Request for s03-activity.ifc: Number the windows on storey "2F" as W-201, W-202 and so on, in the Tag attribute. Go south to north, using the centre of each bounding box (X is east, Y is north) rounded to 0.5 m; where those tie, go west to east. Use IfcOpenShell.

First a look at what the model holds.

```python
import ifcopenshell
import ifcopenshell.util.element
import ifcopenshell.util.placement

model = ifcopenshell.open("s03-activity.ifc")
print(model.schema)
storey = next(s for s in model.by_type("IfcBuildingStorey") if s.Name == "2F")
windows = [e for e in ifcopenshell.util.element.get_decomposition(storey) if e.is_a("IfcWindow")]
for e in sorted(windows, key=lambda e: e.id()):
    origin = ifcopenshell.util.placement.get_local_placement(e.ObjectPlacement)[:3, 3]
    print(e.id(), e.Tag, e.Name, origin.round(2) + 0.0, sep=" | ")
```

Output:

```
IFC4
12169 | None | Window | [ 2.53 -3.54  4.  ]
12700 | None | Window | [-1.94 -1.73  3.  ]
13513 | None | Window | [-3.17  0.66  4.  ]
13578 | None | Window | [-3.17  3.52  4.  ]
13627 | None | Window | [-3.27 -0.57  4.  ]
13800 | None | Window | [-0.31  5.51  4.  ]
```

```python
import ifcopenshell
import ifcopenshell.geom
import ifcopenshell.util.element
import ifcopenshell.util.shape

model = ifcopenshell.open("s03-activity.ifc")
settings = ifcopenshell.geom.settings()
settings.set("use-world-coords", True)


def centre(element):
    shape = ifcopenshell.geom.create_shape(settings, element)
    return ifcopenshell.util.shape.get_bbox_centroid(shape.geometry)


storey = next(s for s in model.by_type("IfcBuildingStorey") if s.Name == "2F")
windows = [e for e in ifcopenshell.util.element.get_decomposition(storey) if e.is_a("IfcWindow")]

# Insertion points can sit at a corner or the storey origin, so sort by the geometry (in metres).
centres = {e: centre(e) for e in windows}
windows.sort(key=lambda e: (round(centres[e][1] / 0.5), centres[e][0]))

for i, e in enumerate(windows, start=1):
    number = f"W-2{i:02d}"
    e.Tag = number
    print(e.id(), number)

model.write("s03-activity_updated.ifc")
```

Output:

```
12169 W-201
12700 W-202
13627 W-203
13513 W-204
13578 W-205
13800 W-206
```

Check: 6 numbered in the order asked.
